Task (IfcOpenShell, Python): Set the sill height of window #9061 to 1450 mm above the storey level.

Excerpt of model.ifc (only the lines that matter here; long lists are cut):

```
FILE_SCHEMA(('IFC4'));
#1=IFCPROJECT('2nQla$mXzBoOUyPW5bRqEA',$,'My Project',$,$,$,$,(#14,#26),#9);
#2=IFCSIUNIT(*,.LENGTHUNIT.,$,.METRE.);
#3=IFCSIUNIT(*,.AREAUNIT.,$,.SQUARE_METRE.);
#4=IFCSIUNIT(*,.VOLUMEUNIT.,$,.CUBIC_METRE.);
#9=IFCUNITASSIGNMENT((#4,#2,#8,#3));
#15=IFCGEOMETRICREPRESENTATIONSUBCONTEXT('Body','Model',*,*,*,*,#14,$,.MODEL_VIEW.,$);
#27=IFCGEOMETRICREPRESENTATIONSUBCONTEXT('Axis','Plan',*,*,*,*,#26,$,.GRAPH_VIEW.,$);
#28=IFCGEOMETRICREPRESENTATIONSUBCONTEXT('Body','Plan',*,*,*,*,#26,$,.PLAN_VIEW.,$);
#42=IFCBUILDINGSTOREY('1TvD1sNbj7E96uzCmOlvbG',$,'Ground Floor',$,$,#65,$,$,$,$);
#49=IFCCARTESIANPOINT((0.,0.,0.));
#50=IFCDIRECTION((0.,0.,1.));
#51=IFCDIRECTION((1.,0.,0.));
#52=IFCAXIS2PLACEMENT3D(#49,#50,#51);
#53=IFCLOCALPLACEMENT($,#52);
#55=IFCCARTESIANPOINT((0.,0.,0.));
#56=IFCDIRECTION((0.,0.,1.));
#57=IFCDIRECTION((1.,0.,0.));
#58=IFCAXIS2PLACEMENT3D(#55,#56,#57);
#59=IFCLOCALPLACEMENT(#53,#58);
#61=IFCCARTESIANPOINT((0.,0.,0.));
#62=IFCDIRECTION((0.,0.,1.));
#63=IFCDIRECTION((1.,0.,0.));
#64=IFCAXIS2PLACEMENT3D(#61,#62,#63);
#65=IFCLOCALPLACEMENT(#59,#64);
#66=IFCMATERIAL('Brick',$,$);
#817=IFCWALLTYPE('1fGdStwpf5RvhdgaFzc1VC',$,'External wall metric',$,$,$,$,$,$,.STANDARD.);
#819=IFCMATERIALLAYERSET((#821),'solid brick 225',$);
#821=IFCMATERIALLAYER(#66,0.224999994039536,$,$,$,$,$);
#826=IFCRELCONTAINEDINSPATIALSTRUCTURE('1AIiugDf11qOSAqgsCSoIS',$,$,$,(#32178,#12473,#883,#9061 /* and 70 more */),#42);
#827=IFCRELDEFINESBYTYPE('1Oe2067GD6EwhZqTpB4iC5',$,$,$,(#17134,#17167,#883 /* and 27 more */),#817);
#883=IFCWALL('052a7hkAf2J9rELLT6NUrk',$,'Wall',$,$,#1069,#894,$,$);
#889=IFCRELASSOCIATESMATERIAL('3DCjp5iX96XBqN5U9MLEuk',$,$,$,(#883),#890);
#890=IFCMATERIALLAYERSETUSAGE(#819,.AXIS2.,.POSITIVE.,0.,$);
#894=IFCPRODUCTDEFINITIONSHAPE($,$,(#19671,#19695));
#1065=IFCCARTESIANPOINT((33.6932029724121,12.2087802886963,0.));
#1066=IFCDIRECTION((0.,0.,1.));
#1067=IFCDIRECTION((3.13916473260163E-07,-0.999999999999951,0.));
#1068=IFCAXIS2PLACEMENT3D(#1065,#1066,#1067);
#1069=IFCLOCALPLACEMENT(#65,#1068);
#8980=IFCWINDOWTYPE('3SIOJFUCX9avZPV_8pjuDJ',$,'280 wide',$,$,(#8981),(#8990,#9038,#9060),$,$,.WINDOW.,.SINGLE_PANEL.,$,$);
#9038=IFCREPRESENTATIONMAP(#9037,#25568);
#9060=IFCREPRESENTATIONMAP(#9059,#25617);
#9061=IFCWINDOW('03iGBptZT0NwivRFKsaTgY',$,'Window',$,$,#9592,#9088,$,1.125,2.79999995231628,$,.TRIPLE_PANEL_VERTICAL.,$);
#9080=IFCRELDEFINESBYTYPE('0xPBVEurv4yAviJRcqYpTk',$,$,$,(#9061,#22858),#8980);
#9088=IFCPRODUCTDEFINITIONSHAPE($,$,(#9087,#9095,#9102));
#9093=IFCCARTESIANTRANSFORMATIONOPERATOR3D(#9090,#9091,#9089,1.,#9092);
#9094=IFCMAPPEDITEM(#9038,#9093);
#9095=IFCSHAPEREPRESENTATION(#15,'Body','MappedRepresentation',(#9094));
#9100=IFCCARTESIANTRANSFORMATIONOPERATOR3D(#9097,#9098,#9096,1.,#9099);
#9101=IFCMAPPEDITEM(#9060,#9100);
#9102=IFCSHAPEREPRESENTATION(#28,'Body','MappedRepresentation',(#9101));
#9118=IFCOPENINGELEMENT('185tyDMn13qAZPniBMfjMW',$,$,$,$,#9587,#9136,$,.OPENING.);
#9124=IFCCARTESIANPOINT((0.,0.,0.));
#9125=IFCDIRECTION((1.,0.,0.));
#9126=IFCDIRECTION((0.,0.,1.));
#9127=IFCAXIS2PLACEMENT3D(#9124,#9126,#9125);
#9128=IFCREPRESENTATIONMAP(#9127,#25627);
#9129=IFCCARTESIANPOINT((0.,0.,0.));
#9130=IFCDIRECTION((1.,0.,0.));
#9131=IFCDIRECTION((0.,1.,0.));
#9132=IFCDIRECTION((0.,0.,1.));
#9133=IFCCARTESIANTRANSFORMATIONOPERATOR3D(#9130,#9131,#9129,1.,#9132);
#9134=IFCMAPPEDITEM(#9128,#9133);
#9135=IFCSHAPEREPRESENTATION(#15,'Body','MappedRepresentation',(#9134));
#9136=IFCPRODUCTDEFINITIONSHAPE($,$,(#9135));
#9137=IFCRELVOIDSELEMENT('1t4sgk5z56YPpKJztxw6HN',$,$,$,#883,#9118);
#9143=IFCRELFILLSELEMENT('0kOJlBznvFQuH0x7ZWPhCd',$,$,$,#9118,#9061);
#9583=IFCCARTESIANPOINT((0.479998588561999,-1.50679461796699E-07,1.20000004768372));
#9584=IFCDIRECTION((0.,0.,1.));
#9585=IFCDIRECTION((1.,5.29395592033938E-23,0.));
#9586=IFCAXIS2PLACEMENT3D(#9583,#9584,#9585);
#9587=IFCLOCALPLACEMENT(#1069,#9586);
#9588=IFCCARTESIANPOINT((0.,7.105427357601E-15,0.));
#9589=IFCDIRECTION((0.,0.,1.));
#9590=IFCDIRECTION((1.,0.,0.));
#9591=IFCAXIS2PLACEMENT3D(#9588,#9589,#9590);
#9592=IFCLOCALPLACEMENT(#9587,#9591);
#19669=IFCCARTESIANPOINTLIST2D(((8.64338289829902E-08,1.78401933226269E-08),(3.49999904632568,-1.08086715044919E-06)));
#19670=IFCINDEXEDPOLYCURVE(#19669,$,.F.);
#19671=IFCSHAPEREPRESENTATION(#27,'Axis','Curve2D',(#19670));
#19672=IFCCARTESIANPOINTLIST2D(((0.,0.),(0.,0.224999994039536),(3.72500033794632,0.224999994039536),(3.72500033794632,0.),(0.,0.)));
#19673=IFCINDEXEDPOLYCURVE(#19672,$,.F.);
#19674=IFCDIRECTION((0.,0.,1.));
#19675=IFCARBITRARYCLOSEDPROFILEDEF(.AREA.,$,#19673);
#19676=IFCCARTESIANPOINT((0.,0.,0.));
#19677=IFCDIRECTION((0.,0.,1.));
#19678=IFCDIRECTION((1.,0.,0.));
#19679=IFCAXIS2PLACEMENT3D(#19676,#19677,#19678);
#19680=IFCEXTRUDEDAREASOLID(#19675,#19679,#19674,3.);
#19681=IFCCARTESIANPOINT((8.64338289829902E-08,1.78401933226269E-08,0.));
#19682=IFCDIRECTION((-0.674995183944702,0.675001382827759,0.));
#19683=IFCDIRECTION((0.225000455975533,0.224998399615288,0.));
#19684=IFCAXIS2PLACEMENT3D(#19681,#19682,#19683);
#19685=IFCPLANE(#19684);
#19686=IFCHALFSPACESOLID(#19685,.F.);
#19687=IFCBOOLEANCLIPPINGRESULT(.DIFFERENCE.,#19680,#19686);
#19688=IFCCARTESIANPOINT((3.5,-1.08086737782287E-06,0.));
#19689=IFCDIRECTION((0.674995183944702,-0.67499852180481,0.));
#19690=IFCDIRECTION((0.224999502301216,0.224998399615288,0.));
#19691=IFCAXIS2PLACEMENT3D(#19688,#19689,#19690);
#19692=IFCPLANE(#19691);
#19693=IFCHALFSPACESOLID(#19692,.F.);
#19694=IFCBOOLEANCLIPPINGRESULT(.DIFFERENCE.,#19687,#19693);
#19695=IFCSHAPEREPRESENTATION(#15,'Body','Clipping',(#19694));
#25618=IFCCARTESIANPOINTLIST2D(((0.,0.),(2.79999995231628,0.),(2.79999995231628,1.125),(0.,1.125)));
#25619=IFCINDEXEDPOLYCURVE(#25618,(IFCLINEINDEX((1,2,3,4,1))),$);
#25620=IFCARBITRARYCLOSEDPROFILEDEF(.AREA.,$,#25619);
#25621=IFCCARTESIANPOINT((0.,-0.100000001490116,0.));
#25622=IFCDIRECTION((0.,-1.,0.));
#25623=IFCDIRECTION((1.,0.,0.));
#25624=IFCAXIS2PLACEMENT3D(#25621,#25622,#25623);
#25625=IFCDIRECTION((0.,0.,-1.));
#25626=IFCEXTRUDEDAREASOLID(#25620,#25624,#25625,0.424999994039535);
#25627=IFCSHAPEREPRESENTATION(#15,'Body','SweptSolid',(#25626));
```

```python
import numpy as np
import ifcopenshell
import ifcopenshell.api.geometry
import ifcopenshell.geom
import ifcopenshell.util.element
import ifcopenshell.util.placement
import ifcopenshell.util.shape
import ifcopenshell.util.unit

model = ifcopenshell.open("model.ifc")
unit_scale = ifcopenshell.util.unit.calculate_unit_scale(model)

window = model.by_id(9061)
opening = window.FillsVoids[0].RelatingOpeningElement
storey = ifcopenshell.util.element.get_container(window, ifc_class="IfcBuildingStorey")
level = ifcopenshell.util.placement.get_local_placement(storey.ObjectPlacement)[2, 3]

# The opening's origin need not be at the sill, so measure its lowest point.
shape = ifcopenshell.geom.create_shape(ifcopenshell.geom.settings(), opening)
bottom = ifcopenshell.util.shape.get_shape_bottom_elevation(shape, shape.geometry) / unit_scale
dz = level + 1.45 / unit_scale - bottom

shift = np.array([0.0, 0.0, dz])
# The window is placed relative to its opening, so it follows when the opening moves.
matrix = ifcopenshell.util.placement.get_local_placement(opening.ObjectPlacement)
matrix[:3, 3] += shift
ifcopenshell.api.geometry.edit_object_placement(
    model, product=opening, matrix=matrix, is_si=False, should_transform_children=True
)

print(f"moved by {dz * unit_scale:+.3f} m")

model.write("model_updated.ifc")
```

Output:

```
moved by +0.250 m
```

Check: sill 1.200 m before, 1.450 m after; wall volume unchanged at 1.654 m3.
